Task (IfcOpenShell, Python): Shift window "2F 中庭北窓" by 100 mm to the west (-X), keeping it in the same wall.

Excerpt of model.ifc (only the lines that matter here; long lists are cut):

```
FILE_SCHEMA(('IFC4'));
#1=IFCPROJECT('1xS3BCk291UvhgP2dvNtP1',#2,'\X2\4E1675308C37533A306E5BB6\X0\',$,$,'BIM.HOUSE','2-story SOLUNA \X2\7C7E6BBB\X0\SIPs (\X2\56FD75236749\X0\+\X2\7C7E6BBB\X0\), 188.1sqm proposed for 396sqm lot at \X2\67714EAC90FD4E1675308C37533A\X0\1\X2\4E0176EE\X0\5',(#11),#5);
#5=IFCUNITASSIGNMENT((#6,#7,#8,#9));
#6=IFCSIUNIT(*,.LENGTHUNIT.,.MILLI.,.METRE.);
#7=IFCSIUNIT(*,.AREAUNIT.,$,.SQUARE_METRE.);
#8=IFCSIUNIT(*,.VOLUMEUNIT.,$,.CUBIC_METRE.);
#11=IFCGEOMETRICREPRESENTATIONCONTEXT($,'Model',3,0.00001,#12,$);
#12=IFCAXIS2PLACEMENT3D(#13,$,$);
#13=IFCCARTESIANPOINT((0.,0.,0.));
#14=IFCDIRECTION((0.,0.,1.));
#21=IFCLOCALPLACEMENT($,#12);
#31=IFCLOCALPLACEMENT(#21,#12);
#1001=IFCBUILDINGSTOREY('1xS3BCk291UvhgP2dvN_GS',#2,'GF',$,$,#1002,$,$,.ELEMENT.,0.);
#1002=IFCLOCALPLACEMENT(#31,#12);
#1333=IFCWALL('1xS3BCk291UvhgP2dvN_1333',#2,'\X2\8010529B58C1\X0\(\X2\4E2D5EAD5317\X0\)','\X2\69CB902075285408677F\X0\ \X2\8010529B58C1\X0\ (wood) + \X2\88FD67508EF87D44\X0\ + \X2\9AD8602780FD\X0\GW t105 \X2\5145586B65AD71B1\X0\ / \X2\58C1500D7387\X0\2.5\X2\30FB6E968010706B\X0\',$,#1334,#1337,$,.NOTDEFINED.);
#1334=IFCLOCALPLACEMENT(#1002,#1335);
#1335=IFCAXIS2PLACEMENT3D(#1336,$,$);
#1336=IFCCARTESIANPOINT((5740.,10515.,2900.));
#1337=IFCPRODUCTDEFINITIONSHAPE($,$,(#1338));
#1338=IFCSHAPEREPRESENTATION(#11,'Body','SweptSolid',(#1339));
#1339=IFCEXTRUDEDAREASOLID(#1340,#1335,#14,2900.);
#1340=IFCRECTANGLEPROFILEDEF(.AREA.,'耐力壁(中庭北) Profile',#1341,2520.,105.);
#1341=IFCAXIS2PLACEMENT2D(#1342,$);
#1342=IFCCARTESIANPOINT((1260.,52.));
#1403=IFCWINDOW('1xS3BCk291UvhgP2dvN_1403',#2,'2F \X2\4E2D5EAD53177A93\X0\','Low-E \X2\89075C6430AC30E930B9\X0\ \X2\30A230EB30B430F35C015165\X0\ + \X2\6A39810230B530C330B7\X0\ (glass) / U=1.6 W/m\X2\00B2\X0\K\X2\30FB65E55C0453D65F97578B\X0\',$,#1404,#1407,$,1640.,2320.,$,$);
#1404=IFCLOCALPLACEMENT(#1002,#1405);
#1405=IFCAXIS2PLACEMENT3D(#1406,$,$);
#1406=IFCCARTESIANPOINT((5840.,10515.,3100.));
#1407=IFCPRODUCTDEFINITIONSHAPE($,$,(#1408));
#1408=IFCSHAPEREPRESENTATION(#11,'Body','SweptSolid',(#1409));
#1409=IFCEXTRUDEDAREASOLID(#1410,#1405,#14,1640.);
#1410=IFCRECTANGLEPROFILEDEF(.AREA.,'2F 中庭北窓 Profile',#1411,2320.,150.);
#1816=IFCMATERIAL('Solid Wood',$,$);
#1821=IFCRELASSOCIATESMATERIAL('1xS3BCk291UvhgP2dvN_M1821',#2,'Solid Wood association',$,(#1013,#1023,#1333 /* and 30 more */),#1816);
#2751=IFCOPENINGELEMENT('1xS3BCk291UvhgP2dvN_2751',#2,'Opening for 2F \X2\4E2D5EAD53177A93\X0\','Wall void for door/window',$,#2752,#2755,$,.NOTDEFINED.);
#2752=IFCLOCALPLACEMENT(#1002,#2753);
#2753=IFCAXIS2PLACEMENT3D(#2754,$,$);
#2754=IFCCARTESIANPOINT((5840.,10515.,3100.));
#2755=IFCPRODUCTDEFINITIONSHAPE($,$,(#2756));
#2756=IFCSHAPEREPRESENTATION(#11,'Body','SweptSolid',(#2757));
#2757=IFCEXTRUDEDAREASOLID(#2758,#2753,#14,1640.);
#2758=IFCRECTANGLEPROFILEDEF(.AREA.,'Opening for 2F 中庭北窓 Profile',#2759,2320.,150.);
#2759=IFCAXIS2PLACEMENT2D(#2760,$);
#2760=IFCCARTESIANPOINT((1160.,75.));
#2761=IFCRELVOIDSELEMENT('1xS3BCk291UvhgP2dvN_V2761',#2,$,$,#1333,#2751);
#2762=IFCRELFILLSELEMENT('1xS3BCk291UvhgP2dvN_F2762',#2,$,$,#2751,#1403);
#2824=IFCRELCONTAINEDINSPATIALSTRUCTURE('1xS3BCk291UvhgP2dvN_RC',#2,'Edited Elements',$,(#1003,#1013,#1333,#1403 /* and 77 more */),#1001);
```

```python
import ifcopenshell
import ifcopenshell.api.geometry
import ifcopenshell.util.placement
import ifcopenshell.util.unit

model = ifcopenshell.open("model.ifc")
unit_scale = ifcopenshell.util.unit.calculate_unit_scale(model)

window = model.by_guid("1xS3BCk291UvhgP2dvN_1403")
opening = window.FillsVoids[0].RelatingOpeningElement
wall = opening.VoidsElements[0].RelatingBuildingElement

wall_matrix = ifcopenshell.util.placement.get_local_placement(wall.ObjectPlacement)
shift = wall_matrix[:3, 0] * -0.1 / unit_scale
before = ifcopenshell.util.placement.get_local_placement(window.ObjectPlacement)[:3, 3].copy()

# The window is not placed relative to its opening, so move both.
for product in (opening, window):
    matrix = ifcopenshell.util.placement.get_local_placement(product.ObjectPlacement)
    matrix[:3, 3] += shift
    ifcopenshell.api.geometry.edit_object_placement(model, product=product, matrix=matrix, is_si=False)

after = ifcopenshell.util.placement.get_local_placement(window.ObjectPlacement)[:3, 3]
print("window moved by", (after - before).round(3) + 0.0)

model.write("model_updated.ifc")
```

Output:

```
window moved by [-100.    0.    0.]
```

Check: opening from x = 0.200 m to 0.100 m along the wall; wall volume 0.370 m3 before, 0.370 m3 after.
